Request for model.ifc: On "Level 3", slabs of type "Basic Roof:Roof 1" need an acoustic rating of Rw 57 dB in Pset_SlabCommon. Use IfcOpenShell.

First a look at what the model holds.

```python
import ifcopenshell
import ifcopenshell.util.element

model = ifcopenshell.open("model.ifc")
print(model.schema)
storey = next(s for s in model.by_type("IfcBuildingStorey") if s.Name == "Level 3")
slabs = [e for e in ifcopenshell.util.element.get_decomposition(storey) if e.is_a("IfcSlab")]
seen = {}
for e in slabs:
    element_type = ifcopenshell.util.element.get_type(e)
    key = (element_type.Name if element_type != e and element_type else None, ifcopenshell.util.element.get_pset(e, "Pset_SlabCommon", "AcousticRating"))
    seen[key] = seen.get(key, 0) + 1
for (name, value), count in sorted(seen.items(), key=str):
    print(count, "x", name, "|", value)
```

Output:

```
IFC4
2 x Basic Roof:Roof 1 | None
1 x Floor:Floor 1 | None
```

```python
import ifcopenshell
import ifcopenshell.api.pset
import ifcopenshell.util.element

model = ifcopenshell.open("model.ifc")

storey = next(s for s in model.by_type("IfcBuildingStorey") if s.Name == "Level 3")
slabs = [e for e in ifcopenshell.util.element.get_decomposition(storey) if e.is_a("IfcSlab")]

count = 0
for e in slabs:
    element_type = ifcopenshell.util.element.get_type(e)
    if element_type in (None, e) or element_type.Name != "Basic Roof:Roof 1":
        continue
    # add_pset returns the element's existing set when there is one.
    pset = ifcopenshell.api.pset.add_pset(model, product=e, name="Pset_SlabCommon")
    ifcopenshell.api.pset.edit_pset(model, pset=pset, properties={"AcousticRating": "Rw 57 dB"})
    count += 1

print(count, "slabs updated")

model.write("model-out.ifc")
```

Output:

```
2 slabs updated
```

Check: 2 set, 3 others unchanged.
